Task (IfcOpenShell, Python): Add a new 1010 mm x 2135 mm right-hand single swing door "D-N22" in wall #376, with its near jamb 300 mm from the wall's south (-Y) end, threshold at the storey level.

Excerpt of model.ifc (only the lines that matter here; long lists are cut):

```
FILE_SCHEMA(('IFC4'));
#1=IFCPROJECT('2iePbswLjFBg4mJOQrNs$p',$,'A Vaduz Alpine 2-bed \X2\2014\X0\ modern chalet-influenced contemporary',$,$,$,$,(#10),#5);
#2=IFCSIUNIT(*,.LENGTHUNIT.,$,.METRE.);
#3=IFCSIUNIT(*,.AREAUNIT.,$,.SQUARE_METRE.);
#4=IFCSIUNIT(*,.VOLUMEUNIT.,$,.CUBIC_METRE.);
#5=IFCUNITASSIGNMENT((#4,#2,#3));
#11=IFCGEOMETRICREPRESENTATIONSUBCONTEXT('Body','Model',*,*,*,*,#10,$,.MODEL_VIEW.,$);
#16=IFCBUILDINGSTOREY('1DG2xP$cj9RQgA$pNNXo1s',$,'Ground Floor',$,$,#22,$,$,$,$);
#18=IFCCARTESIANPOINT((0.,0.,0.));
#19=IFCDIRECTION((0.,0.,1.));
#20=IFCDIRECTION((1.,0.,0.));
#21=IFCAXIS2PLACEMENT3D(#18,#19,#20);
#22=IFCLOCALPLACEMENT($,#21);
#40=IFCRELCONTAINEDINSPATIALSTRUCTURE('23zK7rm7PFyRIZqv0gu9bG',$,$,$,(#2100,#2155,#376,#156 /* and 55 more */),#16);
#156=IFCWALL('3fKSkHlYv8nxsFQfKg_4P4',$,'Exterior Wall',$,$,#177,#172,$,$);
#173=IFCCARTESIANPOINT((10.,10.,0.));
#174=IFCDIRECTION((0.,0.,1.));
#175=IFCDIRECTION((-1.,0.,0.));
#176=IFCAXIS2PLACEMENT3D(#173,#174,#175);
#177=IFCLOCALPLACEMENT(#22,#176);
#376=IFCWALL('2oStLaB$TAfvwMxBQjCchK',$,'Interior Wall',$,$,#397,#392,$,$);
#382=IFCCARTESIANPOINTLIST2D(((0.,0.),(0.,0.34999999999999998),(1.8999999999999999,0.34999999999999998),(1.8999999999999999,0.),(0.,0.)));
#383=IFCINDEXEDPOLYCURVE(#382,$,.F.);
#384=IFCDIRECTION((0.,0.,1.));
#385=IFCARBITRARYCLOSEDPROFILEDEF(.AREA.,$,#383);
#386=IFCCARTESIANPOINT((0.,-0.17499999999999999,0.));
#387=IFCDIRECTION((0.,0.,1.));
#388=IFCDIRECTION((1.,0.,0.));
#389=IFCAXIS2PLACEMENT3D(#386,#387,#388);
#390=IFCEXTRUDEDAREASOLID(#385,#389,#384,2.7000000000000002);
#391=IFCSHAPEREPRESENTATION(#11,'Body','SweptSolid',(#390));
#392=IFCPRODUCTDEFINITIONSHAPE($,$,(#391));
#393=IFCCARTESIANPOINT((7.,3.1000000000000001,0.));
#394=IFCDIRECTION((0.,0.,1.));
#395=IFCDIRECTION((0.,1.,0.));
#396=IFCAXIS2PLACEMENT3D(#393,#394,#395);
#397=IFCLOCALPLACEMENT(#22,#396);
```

```python
import numpy as np
import ifcopenshell
import ifcopenshell.api.feature
import ifcopenshell.api.geometry
import ifcopenshell.api.root
import ifcopenshell.api.spatial
import ifcopenshell.geom
import ifcopenshell.util.element
import ifcopenshell.util.placement
import ifcopenshell.util.representation
import ifcopenshell.util.shape
import ifcopenshell.util.unit

model = ifcopenshell.open("model.ifc")
unit_scale = ifcopenshell.util.unit.calculate_unit_scale(model)
settings = ifcopenshell.geom.settings()


def volume(element):
    """Net volume in cubic metres, openings subtracted."""
    shape = ifcopenshell.geom.create_shape(settings, element)
    return ifcopenshell.util.shape.get_volume(shape.geometry)


wall = model.by_guid("2oStLaB$TAfvwMxBQjCchK")
storey = ifcopenshell.util.element.get_container(wall, ifc_class="IfcBuildingStorey")
context = ifcopenshell.util.representation.get_context(model, "Model", "Body", "MODEL_VIEW")
before = volume(wall)

width, height, from_end, sill = 1.01, 2.135, 0.3, 0.0  # metres

# The wall runs along its own X axis, and the end named is its -X end.
wall_shape = ifcopenshell.geom.create_shape(settings, wall)
x, y, z = ifcopenshell.util.shape.get_vertices(wall_shape.geometry).T
start = x.min() + from_end
face, thickness = float(y.min()), float(y.max() - y.min())
wall_matrix = ifcopenshell.util.placement.get_local_placement(wall.ObjectPlacement)
level = ifcopenshell.util.placement.get_local_placement(storey.ObjectPlacement)[2, 3]


def in_wall(x, y):
    """Placement at x, y metres in the wall's axes, at sill height."""
    matrix = wall_matrix.copy()
    matrix[:, 3] = wall_matrix @ np.array([x / unit_scale, y / unit_scale, 0.0, 1.0])
    matrix[2, 3] = level + sill / unit_scale
    return matrix


# Opening: a box that overshoots both wall faces by 50 mm.
opening = ifcopenshell.api.root.create_entity(model, ifc_class="IfcOpeningElement", predefined_type="OPENING")
box = ifcopenshell.api.geometry.add_wall_representation(
    model, context=context, length=width, height=height, thickness=thickness + 0.1
)
ifcopenshell.api.geometry.assign_representation(model, product=opening, representation=box)
ifcopenshell.api.geometry.edit_object_placement(model, product=opening, matrix=in_wall(start, face - 0.05), is_si=False)
ifcopenshell.api.feature.add_feature(model, feature=opening, element=wall)

door = ifcopenshell.api.root.create_entity(model, ifc_class="IfcDoor", name="D-N22", predefined_type="DOOR")
door.OverallWidth, door.OverallHeight = width / unit_scale, height / unit_scale
door.OperationType = "SINGLE_SWING_RIGHT"
body = ifcopenshell.api.geometry.add_door_representation(
    model,
    context=context,
    overall_width=door.OverallWidth,
    overall_height=door.OverallHeight,
    operation_type="SINGLE_SWING_RIGHT",
    lining_properties={"LiningDepth": thickness / unit_scale, "ThresholdDepth": thickness / unit_scale},
)
ifcopenshell.api.geometry.assign_representation(model, product=door, representation=body)
ifcopenshell.api.spatial.assign_container(model, products=[door], relating_structure=storey)
ifcopenshell.api.feature.add_filling(model, opening=opening, element=door)

# The lining spans the wall, so the door starts at the wall face.
ifcopenshell.api.geometry.edit_object_placement(model, product=door, matrix=in_wall(start, face), is_si=False)

after = volume(wall)

print(f"wall volume {before:.3f} -> {after:.3f} m3")

model.write("model-out.ifc")
```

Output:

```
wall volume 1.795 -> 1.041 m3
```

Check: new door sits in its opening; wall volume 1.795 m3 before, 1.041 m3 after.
